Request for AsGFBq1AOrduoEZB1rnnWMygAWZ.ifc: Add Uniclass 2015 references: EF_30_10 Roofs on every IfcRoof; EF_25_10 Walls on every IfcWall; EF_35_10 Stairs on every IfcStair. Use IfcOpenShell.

First a look at what the model holds.

```python
import ifcopenshell

model = ifcopenshell.open("AsGFBq1AOrduoEZB1rnnWMygAWZ.ifc")
print(model.schema)
print("classifications:", [c.Name for c in model.by_type("IfcClassification")])
for ifc_class in ("IfcDoor", "IfcRoof", "IfcStair", "IfcWall", "IfcWindow"):
    print(ifc_class, len(model.by_type(ifc_class)))
```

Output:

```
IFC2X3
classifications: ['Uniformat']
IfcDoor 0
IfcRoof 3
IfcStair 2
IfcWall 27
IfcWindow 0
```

```python
import ifcopenshell
import ifcopenshell.api.classification

model = ifcopenshell.open("AsGFBq1AOrduoEZB1rnnWMygAWZ.ifc")

# IFC2X3 requires Source and Edition and has no link from the project to the system.
system = model.create_entity("IfcClassification", Source="NBS", Edition="2015", Name="Uniclass 2015")

codes = {
    "IfcRoof": ("EF_30_10", "Roofs"),
    "IfcWall": ("EF_25_10", "Walls"),
    "IfcStair": ("EF_35_10", "Stairs"),
}
for ifc_class, (code, name) in codes.items():
    products = model.by_type(ifc_class)
    ifcopenshell.api.classification.add_reference(
        model, products=products, classification=system, identification=code, name=name
    )
    print(code, len(products))

model.write("AsGFBq1AOrduoEZB1rnnWMygAWZ_updated.ifc")
```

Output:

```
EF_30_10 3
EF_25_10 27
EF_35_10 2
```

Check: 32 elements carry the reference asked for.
